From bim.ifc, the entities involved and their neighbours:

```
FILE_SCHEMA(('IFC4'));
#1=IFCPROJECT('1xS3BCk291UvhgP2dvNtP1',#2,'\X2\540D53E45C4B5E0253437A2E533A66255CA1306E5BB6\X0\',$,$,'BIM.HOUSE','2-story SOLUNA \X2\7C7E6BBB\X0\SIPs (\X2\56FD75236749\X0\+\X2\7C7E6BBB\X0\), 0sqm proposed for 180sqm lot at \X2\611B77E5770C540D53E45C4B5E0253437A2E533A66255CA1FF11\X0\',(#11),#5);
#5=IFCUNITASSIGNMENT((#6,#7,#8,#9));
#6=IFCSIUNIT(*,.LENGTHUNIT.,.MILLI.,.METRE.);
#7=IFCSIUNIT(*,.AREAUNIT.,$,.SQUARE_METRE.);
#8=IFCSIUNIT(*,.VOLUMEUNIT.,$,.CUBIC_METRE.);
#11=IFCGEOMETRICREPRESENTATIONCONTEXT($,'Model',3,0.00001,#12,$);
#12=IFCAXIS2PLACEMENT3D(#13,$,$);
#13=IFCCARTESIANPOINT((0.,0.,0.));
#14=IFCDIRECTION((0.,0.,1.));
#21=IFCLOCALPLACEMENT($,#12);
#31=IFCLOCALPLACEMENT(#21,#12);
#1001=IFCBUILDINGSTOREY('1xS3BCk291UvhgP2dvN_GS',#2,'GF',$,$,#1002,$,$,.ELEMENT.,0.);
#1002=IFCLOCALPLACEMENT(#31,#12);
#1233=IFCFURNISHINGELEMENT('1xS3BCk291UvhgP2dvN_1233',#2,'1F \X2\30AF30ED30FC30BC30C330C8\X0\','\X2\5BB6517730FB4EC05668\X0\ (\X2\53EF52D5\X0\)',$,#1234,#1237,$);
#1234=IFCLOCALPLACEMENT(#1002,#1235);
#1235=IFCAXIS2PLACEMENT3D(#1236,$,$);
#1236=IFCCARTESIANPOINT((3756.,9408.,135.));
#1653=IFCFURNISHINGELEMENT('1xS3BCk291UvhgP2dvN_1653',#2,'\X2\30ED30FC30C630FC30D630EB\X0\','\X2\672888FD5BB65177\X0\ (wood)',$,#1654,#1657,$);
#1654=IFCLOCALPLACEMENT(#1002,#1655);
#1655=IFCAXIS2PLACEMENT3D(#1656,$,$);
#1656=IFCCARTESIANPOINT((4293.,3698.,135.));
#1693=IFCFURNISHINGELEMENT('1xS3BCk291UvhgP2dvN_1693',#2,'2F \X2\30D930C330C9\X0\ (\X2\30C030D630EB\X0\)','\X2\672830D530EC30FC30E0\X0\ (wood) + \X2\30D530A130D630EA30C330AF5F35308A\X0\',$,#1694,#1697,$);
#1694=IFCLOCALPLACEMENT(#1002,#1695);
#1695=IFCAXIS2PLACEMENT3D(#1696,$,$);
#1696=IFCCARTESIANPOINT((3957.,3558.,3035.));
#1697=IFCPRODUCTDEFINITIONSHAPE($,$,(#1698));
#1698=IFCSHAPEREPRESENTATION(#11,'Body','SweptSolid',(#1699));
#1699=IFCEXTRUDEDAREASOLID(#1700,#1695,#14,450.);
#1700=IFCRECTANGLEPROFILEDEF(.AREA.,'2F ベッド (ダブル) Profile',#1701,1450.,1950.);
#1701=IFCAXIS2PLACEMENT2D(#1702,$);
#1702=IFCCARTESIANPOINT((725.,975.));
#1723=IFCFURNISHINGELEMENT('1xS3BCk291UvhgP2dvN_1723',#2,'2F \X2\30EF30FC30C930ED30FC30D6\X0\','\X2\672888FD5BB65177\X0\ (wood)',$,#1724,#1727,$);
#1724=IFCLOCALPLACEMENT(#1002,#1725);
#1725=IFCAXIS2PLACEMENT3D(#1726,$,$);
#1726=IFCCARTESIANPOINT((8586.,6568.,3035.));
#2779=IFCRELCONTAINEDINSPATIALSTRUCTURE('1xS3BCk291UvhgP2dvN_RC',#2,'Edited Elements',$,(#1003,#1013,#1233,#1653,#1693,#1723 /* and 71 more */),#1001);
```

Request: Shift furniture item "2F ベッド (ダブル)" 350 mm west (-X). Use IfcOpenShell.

```python
import ifcopenshell
import ifcopenshell.api.geometry
import ifcopenshell.util.placement
import ifcopenshell.util.unit

model = ifcopenshell.open("bim.ifc")
unit_scale = ifcopenshell.util.unit.calculate_unit_scale(model)

item = model.by_guid("1xS3BCk291UvhgP2dvN_1693")
matrix = ifcopenshell.util.placement.get_local_placement(item.ObjectPlacement)
matrix[0, 3] -= 0.35 / unit_scale
ifcopenshell.api.geometry.edit_object_placement(model, product=item, matrix=matrix, is_si=False)

print(ifcopenshell.util.placement.get_local_placement(item.ObjectPlacement).round(3) + 0.0)

model.write("bim_edited.ifc")
```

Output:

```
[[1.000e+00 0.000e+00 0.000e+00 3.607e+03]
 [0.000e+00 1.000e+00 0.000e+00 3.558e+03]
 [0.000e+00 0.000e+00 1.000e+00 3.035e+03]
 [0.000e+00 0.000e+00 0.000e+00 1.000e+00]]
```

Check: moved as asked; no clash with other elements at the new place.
